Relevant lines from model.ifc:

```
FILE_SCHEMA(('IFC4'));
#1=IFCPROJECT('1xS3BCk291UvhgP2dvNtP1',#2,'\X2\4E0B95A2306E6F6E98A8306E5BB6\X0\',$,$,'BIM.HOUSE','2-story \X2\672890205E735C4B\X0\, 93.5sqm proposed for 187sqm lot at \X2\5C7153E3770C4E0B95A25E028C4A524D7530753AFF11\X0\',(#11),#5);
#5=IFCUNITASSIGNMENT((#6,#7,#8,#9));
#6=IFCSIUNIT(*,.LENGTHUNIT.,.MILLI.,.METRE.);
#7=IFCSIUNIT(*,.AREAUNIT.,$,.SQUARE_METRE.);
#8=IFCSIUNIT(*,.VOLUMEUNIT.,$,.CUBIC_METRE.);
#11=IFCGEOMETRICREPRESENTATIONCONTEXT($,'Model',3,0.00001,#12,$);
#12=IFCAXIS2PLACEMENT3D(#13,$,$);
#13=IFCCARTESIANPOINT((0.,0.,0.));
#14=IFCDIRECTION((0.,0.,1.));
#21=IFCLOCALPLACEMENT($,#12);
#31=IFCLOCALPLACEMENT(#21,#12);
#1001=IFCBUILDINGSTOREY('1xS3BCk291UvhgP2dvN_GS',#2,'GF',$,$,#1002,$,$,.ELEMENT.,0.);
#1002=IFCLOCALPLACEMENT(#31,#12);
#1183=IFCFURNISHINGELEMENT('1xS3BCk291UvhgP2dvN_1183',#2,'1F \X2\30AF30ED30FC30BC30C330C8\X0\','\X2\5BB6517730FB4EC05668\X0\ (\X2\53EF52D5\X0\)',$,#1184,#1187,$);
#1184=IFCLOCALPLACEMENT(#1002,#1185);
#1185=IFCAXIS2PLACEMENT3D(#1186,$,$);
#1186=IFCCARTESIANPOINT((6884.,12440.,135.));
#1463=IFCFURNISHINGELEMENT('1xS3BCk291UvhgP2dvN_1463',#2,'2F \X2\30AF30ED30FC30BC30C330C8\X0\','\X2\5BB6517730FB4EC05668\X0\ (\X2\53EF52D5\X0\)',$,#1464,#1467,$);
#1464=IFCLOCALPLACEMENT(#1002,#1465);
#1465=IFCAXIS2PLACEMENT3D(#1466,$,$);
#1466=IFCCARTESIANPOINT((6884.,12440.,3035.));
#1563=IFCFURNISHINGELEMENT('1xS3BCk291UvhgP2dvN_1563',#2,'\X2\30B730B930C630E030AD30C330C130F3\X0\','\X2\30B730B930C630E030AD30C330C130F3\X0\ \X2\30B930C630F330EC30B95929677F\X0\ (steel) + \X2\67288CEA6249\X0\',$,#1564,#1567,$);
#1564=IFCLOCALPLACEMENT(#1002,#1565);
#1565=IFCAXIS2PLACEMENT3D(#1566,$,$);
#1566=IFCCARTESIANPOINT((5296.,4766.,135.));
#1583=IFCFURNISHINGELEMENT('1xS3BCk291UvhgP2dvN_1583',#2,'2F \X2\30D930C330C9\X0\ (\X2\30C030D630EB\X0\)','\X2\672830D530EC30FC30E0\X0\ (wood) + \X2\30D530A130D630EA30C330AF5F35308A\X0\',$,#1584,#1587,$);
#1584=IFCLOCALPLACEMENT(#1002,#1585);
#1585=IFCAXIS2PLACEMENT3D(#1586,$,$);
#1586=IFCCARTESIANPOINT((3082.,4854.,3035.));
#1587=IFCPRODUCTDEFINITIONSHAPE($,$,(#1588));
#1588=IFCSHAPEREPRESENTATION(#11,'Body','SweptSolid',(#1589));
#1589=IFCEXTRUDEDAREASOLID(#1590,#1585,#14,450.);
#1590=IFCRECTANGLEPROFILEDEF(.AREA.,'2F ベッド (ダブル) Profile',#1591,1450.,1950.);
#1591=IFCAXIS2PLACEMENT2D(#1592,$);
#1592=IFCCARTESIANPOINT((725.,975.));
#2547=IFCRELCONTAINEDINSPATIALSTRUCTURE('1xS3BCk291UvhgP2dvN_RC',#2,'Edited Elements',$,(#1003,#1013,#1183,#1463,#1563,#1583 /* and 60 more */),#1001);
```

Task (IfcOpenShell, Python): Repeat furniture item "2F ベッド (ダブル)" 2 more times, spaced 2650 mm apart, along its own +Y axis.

```python
import ifcopenshell
import ifcopenshell.api.geometry
import ifcopenshell.api.root
import ifcopenshell.util.element
import ifcopenshell.util.placement
import ifcopenshell.util.unit

model = ifcopenshell.open("model.ifc")
unit_scale = ifcopenshell.util.unit.calculate_unit_scale(model)


def reuse_history(source, copy):
    """copy_class also copies each property set's owner history, people and application; keep the originals."""
    for rel in copy.IsDefinedBy:
        if rel.is_a("IfcRelDefinesByProperties") and (history := rel.RelatingPropertyDefinition.OwnerHistory):
            rel.RelatingPropertyDefinition.OwnerHistory = source.OwnerHistory
            ifcopenshell.util.element.remove_deep2(model, history)


source = model.by_id(1583)
base = ifcopenshell.util.placement.get_local_placement(source.ObjectPlacement)
step = base[:3, 1] * 2.65 / unit_scale

for i in range(1, 3):
    copy = ifcopenshell.api.root.copy_class(model, product=source)
    copy.Representation = ifcopenshell.util.element.copy_deep(
        model, source.Representation, exclude=["IfcGeometricRepresentationContext", "IfcRepresentationMap"]
    )
    reuse_history(source, copy)
    matrix = base.copy()
    matrix[:3, 3] += i * step
    print("added at", matrix[:3, 3].round(3) + 0.0)
    ifcopenshell.api.geometry.edit_object_placement(model, product=copy, matrix=matrix, is_si=False)

model.write("model_edited.ifc")
```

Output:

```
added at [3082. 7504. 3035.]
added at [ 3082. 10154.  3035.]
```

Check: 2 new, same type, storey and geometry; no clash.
